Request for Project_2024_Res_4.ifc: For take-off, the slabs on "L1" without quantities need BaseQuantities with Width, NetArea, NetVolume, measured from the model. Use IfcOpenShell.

First a look at what the model holds.

```python
import ifcopenshell
import ifcopenshell.util.element
import ifcopenshell.util.unit

model = ifcopenshell.open("Project_2024_Res_4.ifc")
print(model.schema)
for unit_type in ("LENGTHUNIT", "AREAUNIT", "VOLUMEUNIT"):
    print(unit_type, ifcopenshell.util.unit.calculate_unit_scale(model, unit_type))
storey = next(s for s in model.by_type("IfcBuildingStorey") if s.Name == "L1")
slabs = [e for e in ifcopenshell.util.element.get_decomposition(storey) if e.is_a("IfcSlab")]
for e in sorted(slabs, key=lambda e: e.id()):
    print(e.id(), e.is_a(), e.Name, list(ifcopenshell.util.element.get_psets(e, qtos_only=True)), sep=" | ")
```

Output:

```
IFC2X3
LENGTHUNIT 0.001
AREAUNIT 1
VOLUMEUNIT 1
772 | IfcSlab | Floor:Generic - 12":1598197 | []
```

```python
import ifcopenshell
import ifcopenshell.api.pset
import ifcopenshell.geom
import ifcopenshell.util.element
import ifcopenshell.util.shape
import ifcopenshell.util.unit

model = ifcopenshell.open("Project_2024_Res_4.ifc")
unit_scale = ifcopenshell.util.unit.calculate_unit_scale(model)
area_scale = ifcopenshell.util.unit.calculate_unit_scale(model, "AREAUNIT")
volume_scale = ifcopenshell.util.unit.calculate_unit_scale(model, "VOLUMEUNIT")
settings = ifcopenshell.geom.settings()

storey = next(s for s in model.by_type("IfcBuildingStorey") if s.Name == "L1")
slabs = [e for e in ifcopenshell.util.element.get_decomposition(storey) if e.is_a("IfcSlab")]

for e in sorted(slabs, key=lambda e: e.id()):
    if ifcopenshell.util.element.get_psets(e, qtos_only=True, should_inherit=False):
        continue
    # Geometry comes back in metres, in the element's own axes.
    shape = ifcopenshell.geom.create_shape(settings, e)
    values = {
        "Width": ifcopenshell.util.shape.get_z(shape.geometry) / unit_scale,
        "NetArea": ifcopenshell.util.shape.get_footprint_area(shape.geometry) / area_scale,
        "NetVolume": ifcopenshell.util.shape.get_volume(shape.geometry) / volume_scale,
    }
    qto = ifcopenshell.api.pset.add_qto(model, product=e, name="BaseQuantities")
    ifcopenshell.api.pset.edit_qto(model, qto=qto, properties=values)
    print(e.id(), {k: round(v, 3) for k, v in values.items()})

model.write("Project_2024_Res_4_v2.ifc")
```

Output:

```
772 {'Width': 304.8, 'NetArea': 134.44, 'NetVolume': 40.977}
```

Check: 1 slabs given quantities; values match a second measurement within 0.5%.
